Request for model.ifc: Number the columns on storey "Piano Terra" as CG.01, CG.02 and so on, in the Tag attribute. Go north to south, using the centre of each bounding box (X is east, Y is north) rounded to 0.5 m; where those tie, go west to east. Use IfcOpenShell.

First a look at what the model holds.

```python
import ifcopenshell
import ifcopenshell.util.element
import ifcopenshell.util.placement

model = ifcopenshell.open("model.ifc")
print(model.schema)
storey = next(s for s in model.by_type("IfcBuildingStorey") if s.Name == "Piano Terra")
columns = [e for e in ifcopenshell.util.element.get_decomposition(storey) if e.is_a("IfcColumn")]
for e in sorted(columns, key=lambda e: e.id()):
    origin = ifcopenshell.util.placement.get_local_placement(e.ObjectPlacement)[:3, 3]
    print(e.id(), e.Tag, e.Name, origin.round(2) + 0.0, sep=" | ")
```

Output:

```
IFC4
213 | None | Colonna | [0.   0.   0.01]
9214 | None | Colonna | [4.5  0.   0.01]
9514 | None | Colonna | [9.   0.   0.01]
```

```python
import ifcopenshell
import ifcopenshell.geom
import ifcopenshell.util.element
import ifcopenshell.util.shape

model = ifcopenshell.open("model.ifc")
settings = ifcopenshell.geom.settings()
settings.set("use-world-coords", True)


def centre(element):
    shape = ifcopenshell.geom.create_shape(settings, element)
    return ifcopenshell.util.shape.get_bbox_centroid(shape.geometry)


storey = next(s for s in model.by_type("IfcBuildingStorey") if s.Name == "Piano Terra")
columns = [e for e in ifcopenshell.util.element.get_decomposition(storey) if e.is_a("IfcColumn")]

# Insertion points can sit at a corner or the storey origin, so sort by the geometry (in metres).
centres = {e: centre(e) for e in columns}
columns.sort(key=lambda e: (-round(centres[e][1] / 0.5), centres[e][0]))

for i, e in enumerate(columns, start=1):
    number = f"CG.{i:02d}"
    e.Tag = number
    print(e.id(), number)

model.write("model_rev.ifc")
```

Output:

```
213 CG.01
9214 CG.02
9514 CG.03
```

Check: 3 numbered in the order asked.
